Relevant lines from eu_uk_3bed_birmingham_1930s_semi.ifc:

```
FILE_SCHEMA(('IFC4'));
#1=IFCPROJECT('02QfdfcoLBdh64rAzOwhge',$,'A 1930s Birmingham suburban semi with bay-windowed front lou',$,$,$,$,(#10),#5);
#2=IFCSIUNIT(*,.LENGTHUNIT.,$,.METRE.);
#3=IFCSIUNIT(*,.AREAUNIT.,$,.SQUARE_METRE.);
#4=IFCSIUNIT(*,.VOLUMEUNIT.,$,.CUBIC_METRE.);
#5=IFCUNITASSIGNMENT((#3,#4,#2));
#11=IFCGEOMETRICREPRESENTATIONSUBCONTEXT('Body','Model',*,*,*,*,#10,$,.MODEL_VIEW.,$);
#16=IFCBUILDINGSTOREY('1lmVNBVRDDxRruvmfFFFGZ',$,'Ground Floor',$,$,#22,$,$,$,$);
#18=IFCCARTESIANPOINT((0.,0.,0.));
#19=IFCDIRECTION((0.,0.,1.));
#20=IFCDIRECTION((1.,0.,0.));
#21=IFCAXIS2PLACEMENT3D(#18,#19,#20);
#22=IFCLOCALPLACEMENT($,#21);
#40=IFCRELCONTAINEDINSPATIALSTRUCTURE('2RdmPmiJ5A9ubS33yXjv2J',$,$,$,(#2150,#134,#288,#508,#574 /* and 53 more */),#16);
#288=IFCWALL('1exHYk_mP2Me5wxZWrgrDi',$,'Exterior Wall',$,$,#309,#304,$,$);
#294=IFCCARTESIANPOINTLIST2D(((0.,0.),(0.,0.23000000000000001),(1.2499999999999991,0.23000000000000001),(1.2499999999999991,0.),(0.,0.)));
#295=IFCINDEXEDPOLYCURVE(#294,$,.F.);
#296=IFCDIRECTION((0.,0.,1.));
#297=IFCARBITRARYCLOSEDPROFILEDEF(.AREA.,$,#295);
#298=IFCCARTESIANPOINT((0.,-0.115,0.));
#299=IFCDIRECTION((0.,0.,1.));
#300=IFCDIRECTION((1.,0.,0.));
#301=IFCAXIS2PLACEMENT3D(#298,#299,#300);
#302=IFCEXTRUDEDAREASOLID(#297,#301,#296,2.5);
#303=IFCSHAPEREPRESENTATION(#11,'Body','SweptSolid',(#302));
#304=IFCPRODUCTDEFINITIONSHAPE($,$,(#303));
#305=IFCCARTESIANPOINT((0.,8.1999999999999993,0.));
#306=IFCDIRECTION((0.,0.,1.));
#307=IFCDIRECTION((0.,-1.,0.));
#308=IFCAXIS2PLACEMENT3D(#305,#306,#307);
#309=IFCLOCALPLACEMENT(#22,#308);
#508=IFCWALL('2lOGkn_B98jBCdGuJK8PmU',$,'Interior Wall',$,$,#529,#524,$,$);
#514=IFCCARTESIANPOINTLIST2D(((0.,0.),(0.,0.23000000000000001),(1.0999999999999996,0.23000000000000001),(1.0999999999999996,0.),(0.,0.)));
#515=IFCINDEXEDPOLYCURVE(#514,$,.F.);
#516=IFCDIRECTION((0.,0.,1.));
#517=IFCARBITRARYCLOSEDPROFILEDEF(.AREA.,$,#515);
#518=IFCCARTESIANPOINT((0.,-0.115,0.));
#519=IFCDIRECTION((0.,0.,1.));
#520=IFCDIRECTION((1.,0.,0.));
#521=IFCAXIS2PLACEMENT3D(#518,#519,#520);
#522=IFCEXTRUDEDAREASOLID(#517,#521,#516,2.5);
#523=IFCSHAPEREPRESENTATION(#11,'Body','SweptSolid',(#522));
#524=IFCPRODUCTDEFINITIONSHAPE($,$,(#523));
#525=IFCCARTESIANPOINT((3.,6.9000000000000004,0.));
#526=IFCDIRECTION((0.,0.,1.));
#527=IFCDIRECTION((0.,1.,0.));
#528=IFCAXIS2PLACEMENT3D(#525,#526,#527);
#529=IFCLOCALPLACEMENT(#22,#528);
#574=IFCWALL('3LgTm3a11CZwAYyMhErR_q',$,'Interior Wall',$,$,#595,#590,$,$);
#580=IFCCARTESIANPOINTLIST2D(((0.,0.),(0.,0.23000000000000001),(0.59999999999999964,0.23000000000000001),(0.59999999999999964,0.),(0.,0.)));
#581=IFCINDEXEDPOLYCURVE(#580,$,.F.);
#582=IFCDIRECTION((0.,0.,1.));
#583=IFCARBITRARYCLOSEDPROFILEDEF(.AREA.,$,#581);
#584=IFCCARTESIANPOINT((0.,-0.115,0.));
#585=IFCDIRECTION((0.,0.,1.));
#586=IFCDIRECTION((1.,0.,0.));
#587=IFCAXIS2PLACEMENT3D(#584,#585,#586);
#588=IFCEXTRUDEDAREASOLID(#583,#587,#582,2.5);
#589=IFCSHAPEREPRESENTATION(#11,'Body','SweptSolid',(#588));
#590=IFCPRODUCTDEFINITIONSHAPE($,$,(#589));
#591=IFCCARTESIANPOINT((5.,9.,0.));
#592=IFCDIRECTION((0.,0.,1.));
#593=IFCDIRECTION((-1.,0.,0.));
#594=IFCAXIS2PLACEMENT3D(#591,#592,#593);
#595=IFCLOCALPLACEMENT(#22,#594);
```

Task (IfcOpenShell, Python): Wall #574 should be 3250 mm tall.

```python
import ifcopenshell
import ifcopenshell.geom
import ifcopenshell.util.representation
import ifcopenshell.util.shape
import ifcopenshell.util.unit

model = ifcopenshell.open("eu_uk_3bed_birmingham_1930s_semi.ifc")
unit_scale = ifcopenshell.util.unit.calculate_unit_scale(model)
settings = ifcopenshell.geom.settings()


def volume(element):
    """Net volume in cubic metres, openings subtracted."""
    shape = ifcopenshell.geom.create_shape(settings, element)
    return ifcopenshell.util.shape.get_volume(shape.geometry)


wall = model.by_id(574)
before = volume(wall)

body = ifcopenshell.util.representation.get_representation(wall, "Model", "Body")
solid = body.Items[0]
old_height = solid.Depth
solid.Depth = 3.25 / unit_scale
after = volume(wall)

print(f"height {old_height:g} -> {solid.Depth:g}, volume {before:.3f} -> {after:.3f} m3")

model.write("eu_uk_3bed_birmingham_1930s_semi-out.ifc")
```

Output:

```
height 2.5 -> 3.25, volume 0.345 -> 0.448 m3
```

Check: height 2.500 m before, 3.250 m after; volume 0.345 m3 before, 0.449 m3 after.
